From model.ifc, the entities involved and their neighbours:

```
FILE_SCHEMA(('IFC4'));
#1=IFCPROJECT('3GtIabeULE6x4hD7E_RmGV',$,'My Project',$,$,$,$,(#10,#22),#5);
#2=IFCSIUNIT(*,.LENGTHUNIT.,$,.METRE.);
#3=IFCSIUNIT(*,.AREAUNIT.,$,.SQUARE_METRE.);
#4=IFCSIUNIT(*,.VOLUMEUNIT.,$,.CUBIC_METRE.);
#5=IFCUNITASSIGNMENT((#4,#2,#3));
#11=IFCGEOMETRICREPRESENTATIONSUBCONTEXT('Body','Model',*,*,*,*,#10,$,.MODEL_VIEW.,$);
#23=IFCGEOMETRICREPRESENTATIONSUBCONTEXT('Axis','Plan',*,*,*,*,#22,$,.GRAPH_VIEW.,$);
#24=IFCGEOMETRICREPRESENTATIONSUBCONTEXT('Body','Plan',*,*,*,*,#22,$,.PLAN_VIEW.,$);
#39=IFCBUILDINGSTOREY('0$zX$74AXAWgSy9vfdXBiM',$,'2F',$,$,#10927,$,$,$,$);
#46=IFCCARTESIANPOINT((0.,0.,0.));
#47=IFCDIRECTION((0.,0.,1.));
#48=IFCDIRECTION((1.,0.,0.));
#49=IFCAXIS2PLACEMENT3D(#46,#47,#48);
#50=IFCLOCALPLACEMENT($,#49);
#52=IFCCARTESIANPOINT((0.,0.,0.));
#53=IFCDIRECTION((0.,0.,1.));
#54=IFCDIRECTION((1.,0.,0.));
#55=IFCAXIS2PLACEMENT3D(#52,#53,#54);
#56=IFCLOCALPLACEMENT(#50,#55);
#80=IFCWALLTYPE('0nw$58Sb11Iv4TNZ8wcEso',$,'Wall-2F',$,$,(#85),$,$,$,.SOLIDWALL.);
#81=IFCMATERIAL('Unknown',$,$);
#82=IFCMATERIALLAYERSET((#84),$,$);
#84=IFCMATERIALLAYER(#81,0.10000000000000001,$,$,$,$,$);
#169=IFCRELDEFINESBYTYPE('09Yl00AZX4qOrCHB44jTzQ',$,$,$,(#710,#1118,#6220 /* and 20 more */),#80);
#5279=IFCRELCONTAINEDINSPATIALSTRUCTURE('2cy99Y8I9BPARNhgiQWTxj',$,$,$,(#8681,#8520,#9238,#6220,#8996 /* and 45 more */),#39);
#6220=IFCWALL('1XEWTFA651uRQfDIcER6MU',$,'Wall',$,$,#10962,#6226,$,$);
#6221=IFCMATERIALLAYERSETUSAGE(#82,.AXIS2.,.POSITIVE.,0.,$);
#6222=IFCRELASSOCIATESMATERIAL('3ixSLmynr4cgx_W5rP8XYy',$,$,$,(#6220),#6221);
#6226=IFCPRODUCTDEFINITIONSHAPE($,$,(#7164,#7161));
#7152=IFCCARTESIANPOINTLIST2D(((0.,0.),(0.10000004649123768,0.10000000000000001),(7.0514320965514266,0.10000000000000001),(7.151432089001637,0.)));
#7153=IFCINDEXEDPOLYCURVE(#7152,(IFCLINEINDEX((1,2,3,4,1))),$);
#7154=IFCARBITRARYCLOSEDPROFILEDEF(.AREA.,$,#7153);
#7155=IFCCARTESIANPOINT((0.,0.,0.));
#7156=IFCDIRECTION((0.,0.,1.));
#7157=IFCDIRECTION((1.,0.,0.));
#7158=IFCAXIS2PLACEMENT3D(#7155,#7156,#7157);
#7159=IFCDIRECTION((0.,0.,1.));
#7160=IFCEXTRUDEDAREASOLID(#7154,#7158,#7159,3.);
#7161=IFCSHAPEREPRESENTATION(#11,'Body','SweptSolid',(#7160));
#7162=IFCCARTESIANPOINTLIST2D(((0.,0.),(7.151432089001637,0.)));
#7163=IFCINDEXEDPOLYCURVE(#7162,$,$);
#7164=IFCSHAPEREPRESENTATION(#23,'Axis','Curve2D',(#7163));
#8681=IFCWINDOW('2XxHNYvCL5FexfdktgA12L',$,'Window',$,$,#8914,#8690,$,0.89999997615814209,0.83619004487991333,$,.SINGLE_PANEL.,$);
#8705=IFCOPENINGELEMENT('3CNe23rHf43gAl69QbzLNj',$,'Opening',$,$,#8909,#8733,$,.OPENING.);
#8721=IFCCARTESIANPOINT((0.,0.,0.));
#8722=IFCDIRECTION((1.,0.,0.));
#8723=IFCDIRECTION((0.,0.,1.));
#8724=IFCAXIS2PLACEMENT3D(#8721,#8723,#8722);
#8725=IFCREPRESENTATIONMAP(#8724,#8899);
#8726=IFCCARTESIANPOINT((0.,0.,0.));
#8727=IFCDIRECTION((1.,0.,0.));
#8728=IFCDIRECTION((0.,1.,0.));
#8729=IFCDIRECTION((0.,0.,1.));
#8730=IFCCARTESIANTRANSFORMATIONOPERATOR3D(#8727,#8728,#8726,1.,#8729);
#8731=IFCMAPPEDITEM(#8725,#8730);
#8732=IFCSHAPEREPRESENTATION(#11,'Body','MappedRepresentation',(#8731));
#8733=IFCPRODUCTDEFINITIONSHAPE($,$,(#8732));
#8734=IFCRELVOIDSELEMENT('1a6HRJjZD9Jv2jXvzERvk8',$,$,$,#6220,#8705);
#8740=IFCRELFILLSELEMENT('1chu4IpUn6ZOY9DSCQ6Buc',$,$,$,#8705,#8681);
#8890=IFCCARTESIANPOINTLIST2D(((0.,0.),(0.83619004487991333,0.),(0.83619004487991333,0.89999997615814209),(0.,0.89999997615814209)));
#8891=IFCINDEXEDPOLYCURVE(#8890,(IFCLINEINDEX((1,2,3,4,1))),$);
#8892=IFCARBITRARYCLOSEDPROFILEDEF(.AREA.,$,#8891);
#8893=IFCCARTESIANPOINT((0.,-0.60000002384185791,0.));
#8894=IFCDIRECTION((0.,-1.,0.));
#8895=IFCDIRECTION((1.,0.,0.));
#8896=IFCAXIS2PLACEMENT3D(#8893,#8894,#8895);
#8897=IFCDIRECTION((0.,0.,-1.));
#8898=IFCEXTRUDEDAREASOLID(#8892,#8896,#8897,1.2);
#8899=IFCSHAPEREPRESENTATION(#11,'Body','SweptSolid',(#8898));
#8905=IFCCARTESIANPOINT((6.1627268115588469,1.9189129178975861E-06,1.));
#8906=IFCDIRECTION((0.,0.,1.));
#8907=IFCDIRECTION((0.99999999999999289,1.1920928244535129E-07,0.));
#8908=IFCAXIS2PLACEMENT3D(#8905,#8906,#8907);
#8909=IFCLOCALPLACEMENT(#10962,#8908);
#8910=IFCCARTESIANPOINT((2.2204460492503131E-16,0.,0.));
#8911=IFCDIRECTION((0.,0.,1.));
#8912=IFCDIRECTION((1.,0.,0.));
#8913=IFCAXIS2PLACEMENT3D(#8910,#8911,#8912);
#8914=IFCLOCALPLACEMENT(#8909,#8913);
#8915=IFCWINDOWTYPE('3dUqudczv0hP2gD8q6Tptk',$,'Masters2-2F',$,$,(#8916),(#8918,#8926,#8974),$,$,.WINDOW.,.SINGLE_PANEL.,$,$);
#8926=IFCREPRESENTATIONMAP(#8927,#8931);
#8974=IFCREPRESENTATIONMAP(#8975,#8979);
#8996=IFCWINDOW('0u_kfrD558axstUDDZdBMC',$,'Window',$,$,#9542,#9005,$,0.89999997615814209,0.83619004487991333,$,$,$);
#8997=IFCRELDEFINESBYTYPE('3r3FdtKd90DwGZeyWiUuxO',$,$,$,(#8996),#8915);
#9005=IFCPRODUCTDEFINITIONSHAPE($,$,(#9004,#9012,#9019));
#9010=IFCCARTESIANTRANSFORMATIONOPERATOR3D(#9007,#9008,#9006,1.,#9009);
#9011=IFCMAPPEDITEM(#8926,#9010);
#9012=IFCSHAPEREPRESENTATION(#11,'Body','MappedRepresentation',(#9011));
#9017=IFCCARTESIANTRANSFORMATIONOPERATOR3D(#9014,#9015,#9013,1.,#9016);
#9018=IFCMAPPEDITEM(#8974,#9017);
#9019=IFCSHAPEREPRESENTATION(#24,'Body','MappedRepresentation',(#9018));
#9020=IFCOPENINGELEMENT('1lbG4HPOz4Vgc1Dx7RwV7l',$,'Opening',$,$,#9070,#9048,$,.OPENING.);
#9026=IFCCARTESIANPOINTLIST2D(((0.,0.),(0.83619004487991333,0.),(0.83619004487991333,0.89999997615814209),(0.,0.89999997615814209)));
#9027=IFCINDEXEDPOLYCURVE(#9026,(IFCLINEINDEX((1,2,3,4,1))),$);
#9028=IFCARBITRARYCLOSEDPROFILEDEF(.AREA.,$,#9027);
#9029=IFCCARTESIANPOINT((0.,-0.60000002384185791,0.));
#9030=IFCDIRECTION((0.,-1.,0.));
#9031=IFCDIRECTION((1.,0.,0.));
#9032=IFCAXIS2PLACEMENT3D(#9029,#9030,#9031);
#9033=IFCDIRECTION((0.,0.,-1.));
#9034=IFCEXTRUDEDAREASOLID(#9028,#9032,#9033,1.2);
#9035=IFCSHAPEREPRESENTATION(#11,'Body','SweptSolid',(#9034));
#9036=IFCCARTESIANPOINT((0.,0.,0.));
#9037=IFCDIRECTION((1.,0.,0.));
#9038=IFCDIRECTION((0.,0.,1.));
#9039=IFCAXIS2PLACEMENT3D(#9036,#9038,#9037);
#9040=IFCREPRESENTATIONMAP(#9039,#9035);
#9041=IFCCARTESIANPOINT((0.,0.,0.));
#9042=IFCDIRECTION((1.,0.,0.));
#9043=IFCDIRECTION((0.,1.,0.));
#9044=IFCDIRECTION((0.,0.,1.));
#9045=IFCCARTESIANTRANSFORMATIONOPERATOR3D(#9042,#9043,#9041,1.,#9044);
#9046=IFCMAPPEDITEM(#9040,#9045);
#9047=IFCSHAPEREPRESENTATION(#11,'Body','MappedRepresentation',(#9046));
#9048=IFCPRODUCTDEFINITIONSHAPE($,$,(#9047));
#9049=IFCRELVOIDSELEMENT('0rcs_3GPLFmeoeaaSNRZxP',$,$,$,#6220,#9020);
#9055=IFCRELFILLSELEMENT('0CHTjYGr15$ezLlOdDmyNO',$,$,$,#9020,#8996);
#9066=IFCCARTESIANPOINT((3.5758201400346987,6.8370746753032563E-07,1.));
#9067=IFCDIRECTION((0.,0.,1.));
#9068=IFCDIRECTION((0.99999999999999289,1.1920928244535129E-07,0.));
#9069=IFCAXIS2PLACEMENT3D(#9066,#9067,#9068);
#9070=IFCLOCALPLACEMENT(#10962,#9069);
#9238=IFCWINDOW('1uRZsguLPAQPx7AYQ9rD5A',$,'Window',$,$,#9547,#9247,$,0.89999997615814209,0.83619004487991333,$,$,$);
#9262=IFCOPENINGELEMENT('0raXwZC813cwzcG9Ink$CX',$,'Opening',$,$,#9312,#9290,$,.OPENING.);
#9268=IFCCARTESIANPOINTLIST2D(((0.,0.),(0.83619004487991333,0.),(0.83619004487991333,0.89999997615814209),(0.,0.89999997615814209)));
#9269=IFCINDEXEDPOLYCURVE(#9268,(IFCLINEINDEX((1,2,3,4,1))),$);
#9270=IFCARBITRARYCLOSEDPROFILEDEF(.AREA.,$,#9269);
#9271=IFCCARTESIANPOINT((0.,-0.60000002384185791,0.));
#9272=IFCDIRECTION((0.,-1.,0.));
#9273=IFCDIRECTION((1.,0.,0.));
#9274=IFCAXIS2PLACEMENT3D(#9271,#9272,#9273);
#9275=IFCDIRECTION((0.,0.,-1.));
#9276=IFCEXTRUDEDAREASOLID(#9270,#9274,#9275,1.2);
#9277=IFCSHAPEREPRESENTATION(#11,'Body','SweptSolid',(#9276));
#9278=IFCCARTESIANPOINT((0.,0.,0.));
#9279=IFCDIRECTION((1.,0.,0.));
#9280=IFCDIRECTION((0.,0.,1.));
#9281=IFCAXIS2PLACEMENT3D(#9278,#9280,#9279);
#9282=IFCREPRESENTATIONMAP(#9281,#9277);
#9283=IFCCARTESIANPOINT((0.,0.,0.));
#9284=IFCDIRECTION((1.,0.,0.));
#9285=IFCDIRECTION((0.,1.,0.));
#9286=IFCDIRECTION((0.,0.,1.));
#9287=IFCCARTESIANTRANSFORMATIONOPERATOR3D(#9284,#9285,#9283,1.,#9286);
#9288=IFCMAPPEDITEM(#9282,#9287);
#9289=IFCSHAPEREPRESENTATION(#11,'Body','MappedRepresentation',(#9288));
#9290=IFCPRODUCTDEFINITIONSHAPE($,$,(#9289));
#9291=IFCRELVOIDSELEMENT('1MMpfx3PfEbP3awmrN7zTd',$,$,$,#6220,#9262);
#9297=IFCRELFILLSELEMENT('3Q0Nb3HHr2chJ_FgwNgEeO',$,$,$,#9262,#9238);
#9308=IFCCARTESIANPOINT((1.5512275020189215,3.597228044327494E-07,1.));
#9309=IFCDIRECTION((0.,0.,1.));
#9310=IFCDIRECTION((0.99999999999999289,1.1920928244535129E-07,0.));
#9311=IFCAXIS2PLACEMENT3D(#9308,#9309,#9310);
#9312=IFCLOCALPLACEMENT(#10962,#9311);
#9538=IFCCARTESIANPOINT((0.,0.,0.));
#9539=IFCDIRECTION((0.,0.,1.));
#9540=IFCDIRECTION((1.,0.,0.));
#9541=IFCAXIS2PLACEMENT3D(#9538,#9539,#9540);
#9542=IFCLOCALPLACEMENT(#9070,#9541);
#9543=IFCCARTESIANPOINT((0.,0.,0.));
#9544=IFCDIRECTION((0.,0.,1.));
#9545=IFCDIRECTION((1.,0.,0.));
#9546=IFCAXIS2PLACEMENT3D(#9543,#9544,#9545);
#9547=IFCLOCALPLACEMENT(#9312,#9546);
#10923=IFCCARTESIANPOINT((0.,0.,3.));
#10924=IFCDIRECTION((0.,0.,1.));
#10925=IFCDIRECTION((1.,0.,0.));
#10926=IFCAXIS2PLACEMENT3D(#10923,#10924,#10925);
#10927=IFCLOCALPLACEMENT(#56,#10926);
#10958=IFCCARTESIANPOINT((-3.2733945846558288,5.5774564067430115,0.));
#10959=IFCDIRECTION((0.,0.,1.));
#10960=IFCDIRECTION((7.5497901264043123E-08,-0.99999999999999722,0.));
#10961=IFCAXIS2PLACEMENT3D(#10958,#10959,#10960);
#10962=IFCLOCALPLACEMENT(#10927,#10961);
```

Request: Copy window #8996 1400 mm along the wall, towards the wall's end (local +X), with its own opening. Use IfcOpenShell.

```python
import ifcopenshell
import ifcopenshell.api.feature
import ifcopenshell.api.geometry
import ifcopenshell.api.root
import ifcopenshell.geom
import ifcopenshell.util.element
import ifcopenshell.util.placement
import ifcopenshell.util.shape

model = ifcopenshell.open("model.ifc")
settings = ifcopenshell.geom.settings()


def volume(element):
    """Net volume in cubic metres, openings subtracted."""
    shape = ifcopenshell.geom.create_shape(settings, element)
    return ifcopenshell.util.shape.get_volume(shape.geometry)


window = model.by_id(8996)
opening = window.FillsVoids[0].RelatingOpeningElement
wall = opening.VoidsElements[0].RelatingBuildingElement
before = volume(wall)
shift = ifcopenshell.util.placement.get_local_placement(wall.ObjectPlacement)[:3, 0] * 1.4

# copy_class copies the void relationship, type, container and properties, but no geometry.
new_opening = ifcopenshell.api.root.copy_class(model, product=opening)
new_opening.Representation = ifcopenshell.util.element.copy_deep(
    model, opening.Representation, exclude=["IfcGeometricRepresentationContext", "IfcRepresentationMap"]
)
new_window = ifcopenshell.api.root.copy_class(model, product=window)
new_window.Representation = ifcopenshell.util.element.copy_deep(
    model, window.Representation, exclude=["IfcGeometricRepresentationContext", "IfcRepresentationMap"]
)
ifcopenshell.api.feature.add_filling(model, opening=new_opening, element=new_window)

for old, new in ((opening, new_opening), (window, new_window)):
    matrix = ifcopenshell.util.placement.get_local_placement(old.ObjectPlacement)
    matrix[:3, 3] += shift
    ifcopenshell.api.geometry.edit_object_placement(model, product=new, matrix=matrix, is_si=False)

after = volume(wall)

print(f"wall volume {before:.3f} -> {after:.3f} m3")

model.write("model_updated.ifc")
```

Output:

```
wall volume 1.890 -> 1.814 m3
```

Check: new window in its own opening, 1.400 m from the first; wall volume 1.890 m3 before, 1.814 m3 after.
